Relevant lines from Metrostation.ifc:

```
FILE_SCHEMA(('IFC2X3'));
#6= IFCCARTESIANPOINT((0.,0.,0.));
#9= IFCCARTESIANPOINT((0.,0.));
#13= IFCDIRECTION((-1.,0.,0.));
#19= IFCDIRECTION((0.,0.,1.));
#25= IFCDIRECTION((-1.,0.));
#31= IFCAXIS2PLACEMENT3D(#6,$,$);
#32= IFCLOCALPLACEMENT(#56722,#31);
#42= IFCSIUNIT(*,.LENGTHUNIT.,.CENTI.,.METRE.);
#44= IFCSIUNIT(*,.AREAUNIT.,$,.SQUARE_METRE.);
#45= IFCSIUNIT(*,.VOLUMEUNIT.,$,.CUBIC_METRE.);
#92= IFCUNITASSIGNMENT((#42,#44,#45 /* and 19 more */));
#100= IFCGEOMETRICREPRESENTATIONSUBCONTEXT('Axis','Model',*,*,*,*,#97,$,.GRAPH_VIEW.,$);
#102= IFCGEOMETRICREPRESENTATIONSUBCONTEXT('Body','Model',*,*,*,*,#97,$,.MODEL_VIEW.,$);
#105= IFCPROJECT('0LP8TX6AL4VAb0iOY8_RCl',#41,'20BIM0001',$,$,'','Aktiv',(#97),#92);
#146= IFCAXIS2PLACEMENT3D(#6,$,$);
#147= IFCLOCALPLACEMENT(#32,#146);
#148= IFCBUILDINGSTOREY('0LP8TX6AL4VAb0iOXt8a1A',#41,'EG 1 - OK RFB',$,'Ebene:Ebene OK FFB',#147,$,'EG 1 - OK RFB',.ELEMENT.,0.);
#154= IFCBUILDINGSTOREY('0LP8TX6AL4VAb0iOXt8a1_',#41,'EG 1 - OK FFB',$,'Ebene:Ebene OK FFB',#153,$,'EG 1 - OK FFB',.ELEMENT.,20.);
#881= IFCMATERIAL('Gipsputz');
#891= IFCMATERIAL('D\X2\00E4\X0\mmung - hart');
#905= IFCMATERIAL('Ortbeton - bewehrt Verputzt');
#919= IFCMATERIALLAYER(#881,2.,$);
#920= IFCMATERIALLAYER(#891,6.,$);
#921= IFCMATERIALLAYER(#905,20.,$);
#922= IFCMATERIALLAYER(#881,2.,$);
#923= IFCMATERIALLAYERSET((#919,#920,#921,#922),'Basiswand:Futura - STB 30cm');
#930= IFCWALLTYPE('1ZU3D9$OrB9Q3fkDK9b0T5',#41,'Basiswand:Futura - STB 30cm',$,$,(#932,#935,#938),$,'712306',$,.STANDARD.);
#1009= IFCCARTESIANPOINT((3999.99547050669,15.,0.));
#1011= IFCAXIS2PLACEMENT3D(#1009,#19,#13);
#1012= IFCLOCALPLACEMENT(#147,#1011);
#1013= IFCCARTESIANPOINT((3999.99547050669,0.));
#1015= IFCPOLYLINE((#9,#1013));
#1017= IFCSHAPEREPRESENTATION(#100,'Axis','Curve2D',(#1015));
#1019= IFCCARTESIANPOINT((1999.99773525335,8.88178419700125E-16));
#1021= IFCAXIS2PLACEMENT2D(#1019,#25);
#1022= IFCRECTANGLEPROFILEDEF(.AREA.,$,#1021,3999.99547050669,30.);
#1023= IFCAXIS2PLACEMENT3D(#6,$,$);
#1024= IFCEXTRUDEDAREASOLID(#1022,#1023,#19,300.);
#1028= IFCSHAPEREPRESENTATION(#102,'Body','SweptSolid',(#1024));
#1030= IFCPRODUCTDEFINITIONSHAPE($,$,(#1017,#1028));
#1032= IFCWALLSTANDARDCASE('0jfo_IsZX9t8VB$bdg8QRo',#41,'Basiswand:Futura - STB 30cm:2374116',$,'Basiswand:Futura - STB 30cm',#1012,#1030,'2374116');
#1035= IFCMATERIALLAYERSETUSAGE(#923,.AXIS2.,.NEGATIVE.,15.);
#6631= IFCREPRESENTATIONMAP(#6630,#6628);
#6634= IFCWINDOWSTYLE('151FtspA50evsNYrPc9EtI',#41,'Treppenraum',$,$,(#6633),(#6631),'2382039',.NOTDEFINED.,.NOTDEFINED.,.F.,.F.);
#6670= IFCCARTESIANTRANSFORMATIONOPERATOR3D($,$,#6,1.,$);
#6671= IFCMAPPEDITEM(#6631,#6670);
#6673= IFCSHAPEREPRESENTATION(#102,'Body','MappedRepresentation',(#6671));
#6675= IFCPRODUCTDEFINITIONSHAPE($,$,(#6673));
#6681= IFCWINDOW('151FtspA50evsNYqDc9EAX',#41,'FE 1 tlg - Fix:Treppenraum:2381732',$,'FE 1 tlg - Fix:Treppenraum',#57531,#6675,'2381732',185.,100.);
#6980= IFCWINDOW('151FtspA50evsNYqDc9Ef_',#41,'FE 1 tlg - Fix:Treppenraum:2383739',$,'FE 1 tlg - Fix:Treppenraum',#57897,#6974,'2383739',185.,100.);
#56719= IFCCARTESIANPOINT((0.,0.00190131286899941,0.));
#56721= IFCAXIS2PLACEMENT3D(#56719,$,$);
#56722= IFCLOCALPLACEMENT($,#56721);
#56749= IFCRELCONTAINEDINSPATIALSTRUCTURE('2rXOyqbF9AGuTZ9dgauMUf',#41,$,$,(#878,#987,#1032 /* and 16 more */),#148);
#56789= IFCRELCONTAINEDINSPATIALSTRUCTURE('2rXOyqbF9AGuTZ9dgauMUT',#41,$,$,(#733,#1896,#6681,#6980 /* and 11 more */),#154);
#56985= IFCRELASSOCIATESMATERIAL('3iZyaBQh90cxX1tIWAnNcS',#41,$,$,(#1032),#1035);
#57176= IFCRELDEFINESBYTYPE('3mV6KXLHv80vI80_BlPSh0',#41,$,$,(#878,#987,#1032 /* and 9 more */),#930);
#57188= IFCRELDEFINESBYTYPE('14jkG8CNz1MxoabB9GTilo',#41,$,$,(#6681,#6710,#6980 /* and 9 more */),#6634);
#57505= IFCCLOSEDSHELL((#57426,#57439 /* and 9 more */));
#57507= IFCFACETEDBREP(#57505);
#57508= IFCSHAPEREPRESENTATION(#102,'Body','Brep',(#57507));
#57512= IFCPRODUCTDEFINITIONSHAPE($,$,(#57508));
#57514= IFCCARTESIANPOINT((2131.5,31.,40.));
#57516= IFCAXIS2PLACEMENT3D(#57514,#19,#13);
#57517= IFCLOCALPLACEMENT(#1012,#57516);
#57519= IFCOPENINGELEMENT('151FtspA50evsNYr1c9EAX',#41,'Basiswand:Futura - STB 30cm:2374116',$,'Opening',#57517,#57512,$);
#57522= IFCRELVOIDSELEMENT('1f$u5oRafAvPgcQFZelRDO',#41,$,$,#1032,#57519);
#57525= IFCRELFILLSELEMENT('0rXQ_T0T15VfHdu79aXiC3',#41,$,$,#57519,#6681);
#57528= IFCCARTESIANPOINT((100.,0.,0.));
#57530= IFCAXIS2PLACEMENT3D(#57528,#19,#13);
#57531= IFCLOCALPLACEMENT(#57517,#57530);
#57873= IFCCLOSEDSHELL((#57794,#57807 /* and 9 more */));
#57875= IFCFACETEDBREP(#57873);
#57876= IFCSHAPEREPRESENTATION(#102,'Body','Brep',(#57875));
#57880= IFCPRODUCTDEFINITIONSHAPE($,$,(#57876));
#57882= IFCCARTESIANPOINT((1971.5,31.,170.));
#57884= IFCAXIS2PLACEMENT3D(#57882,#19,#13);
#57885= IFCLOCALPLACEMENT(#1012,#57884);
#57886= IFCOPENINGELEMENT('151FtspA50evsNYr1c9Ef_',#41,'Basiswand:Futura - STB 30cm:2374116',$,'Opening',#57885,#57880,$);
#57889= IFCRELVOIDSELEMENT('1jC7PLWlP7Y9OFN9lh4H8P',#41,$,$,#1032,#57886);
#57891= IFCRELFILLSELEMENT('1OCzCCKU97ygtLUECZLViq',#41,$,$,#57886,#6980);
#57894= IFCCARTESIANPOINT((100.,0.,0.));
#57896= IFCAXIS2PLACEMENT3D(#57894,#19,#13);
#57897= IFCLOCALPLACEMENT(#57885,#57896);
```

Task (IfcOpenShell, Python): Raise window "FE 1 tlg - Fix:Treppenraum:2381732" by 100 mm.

```python
import numpy as np
import ifcopenshell
import ifcopenshell.api.geometry
import ifcopenshell.util.placement
import ifcopenshell.util.unit

model = ifcopenshell.open("Metrostation.ifc")
unit_scale = ifcopenshell.util.unit.calculate_unit_scale(model)

window = model.by_id(6681)
opening = window.FillsVoids[0].RelatingOpeningElement
dz = 0.1 / unit_scale

shift = np.array([0.0, 0.0, dz])
# The window is placed relative to its opening, so it follows when the opening moves.
matrix = ifcopenshell.util.placement.get_local_placement(opening.ObjectPlacement)
matrix[:3, 3] += shift
ifcopenshell.api.geometry.edit_object_placement(
    model, product=opening, matrix=matrix, is_si=False, should_transform_children=True
)

print(f"moved by {dz * unit_scale:+.3f} m")

model.write("Metrostation_rev.ifc")
```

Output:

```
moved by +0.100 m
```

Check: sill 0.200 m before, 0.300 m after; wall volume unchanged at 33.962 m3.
